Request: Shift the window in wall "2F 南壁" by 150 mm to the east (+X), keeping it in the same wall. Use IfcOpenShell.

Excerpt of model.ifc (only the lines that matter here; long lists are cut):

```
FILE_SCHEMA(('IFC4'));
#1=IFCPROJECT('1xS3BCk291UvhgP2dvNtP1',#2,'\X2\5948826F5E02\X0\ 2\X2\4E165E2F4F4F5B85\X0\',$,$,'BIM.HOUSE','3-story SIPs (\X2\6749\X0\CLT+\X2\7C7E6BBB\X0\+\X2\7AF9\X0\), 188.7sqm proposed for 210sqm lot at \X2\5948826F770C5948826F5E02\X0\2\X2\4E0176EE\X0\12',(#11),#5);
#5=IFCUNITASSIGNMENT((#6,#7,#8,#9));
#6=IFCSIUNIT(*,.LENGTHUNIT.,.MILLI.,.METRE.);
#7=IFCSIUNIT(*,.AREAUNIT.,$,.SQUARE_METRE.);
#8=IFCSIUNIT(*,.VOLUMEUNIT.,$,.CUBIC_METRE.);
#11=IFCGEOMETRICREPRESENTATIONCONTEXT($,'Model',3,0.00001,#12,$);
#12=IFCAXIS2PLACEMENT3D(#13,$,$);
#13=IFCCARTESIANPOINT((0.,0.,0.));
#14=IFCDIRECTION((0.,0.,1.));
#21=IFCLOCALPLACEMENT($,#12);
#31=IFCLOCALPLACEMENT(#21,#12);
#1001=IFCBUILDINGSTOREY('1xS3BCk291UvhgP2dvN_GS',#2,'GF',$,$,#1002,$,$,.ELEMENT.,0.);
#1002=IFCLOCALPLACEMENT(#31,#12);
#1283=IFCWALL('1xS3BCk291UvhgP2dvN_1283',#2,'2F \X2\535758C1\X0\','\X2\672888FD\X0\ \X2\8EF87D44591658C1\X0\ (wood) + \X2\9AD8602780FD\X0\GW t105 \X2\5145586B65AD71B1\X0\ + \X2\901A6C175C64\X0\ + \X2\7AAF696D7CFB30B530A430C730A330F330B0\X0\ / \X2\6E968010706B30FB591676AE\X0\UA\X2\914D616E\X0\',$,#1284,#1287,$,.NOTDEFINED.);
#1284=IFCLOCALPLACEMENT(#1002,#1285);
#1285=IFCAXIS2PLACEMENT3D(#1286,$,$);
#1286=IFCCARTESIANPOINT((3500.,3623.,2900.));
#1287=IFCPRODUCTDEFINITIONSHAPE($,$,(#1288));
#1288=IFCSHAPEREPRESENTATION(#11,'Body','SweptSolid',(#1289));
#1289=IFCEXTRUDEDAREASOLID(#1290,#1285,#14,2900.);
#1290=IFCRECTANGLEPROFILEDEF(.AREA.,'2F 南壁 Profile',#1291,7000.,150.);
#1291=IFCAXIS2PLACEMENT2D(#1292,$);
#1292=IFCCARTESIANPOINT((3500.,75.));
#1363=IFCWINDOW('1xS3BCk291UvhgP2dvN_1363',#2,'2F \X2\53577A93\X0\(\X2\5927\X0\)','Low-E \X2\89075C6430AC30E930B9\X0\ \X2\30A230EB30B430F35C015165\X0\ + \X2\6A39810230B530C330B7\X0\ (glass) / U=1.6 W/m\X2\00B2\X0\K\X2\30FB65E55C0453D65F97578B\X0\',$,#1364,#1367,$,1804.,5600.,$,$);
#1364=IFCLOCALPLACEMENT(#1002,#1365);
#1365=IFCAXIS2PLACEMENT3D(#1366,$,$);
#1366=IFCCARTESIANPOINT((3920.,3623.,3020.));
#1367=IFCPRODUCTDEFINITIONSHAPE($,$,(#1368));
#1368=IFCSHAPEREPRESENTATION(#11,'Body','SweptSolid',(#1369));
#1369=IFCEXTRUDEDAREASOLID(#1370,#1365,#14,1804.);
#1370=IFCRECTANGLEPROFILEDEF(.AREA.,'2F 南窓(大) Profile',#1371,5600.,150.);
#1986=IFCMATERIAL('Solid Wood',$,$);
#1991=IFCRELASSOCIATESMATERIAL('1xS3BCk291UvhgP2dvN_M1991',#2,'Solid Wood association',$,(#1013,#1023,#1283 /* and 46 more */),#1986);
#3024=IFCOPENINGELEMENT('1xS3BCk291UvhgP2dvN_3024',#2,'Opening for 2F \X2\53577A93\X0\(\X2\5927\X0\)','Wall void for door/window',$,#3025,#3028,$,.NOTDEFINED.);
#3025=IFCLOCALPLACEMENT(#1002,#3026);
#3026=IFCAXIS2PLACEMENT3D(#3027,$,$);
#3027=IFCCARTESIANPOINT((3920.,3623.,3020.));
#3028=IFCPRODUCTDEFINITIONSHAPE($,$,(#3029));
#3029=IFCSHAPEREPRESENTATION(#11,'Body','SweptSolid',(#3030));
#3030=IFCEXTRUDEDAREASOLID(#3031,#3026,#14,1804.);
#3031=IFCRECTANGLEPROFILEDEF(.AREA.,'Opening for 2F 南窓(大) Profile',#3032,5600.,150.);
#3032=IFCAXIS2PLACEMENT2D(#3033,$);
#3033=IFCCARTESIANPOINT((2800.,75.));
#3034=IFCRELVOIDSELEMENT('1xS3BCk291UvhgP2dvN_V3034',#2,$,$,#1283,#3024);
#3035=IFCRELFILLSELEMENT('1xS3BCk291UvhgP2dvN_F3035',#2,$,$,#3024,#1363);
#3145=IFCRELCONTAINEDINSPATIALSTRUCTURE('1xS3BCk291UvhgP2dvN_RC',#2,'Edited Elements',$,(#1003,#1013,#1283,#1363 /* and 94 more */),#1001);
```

```python
import ifcopenshell
import ifcopenshell.api.geometry
import ifcopenshell.util.placement

model = ifcopenshell.open("model.ifc")

window = model.by_guid("1xS3BCk291UvhgP2dvN_1363")
opening = window.FillsVoids[0].RelatingOpeningElement
wall = opening.VoidsElements[0].RelatingBuildingElement

wall_matrix = ifcopenshell.util.placement.get_local_placement(wall.ObjectPlacement)
shift = wall_matrix[:3, 0] * 150.0
before = ifcopenshell.util.placement.get_local_placement(window.ObjectPlacement)[:3, 3].copy()

# The window is not placed relative to its opening, so move both.
for product in (opening, window):
    matrix = ifcopenshell.util.placement.get_local_placement(product.ObjectPlacement)
    matrix[:3, 3] += shift
    ifcopenshell.api.geometry.edit_object_placement(model, product=product, matrix=matrix, is_si=False)

after = ifcopenshell.util.placement.get_local_placement(window.ObjectPlacement)[:3, 3]
print("window moved by", (after - before).round(3) + 0.0)

model.write("model_v2.ifc")
```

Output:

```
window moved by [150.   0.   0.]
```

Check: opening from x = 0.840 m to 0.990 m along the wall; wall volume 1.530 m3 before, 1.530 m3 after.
